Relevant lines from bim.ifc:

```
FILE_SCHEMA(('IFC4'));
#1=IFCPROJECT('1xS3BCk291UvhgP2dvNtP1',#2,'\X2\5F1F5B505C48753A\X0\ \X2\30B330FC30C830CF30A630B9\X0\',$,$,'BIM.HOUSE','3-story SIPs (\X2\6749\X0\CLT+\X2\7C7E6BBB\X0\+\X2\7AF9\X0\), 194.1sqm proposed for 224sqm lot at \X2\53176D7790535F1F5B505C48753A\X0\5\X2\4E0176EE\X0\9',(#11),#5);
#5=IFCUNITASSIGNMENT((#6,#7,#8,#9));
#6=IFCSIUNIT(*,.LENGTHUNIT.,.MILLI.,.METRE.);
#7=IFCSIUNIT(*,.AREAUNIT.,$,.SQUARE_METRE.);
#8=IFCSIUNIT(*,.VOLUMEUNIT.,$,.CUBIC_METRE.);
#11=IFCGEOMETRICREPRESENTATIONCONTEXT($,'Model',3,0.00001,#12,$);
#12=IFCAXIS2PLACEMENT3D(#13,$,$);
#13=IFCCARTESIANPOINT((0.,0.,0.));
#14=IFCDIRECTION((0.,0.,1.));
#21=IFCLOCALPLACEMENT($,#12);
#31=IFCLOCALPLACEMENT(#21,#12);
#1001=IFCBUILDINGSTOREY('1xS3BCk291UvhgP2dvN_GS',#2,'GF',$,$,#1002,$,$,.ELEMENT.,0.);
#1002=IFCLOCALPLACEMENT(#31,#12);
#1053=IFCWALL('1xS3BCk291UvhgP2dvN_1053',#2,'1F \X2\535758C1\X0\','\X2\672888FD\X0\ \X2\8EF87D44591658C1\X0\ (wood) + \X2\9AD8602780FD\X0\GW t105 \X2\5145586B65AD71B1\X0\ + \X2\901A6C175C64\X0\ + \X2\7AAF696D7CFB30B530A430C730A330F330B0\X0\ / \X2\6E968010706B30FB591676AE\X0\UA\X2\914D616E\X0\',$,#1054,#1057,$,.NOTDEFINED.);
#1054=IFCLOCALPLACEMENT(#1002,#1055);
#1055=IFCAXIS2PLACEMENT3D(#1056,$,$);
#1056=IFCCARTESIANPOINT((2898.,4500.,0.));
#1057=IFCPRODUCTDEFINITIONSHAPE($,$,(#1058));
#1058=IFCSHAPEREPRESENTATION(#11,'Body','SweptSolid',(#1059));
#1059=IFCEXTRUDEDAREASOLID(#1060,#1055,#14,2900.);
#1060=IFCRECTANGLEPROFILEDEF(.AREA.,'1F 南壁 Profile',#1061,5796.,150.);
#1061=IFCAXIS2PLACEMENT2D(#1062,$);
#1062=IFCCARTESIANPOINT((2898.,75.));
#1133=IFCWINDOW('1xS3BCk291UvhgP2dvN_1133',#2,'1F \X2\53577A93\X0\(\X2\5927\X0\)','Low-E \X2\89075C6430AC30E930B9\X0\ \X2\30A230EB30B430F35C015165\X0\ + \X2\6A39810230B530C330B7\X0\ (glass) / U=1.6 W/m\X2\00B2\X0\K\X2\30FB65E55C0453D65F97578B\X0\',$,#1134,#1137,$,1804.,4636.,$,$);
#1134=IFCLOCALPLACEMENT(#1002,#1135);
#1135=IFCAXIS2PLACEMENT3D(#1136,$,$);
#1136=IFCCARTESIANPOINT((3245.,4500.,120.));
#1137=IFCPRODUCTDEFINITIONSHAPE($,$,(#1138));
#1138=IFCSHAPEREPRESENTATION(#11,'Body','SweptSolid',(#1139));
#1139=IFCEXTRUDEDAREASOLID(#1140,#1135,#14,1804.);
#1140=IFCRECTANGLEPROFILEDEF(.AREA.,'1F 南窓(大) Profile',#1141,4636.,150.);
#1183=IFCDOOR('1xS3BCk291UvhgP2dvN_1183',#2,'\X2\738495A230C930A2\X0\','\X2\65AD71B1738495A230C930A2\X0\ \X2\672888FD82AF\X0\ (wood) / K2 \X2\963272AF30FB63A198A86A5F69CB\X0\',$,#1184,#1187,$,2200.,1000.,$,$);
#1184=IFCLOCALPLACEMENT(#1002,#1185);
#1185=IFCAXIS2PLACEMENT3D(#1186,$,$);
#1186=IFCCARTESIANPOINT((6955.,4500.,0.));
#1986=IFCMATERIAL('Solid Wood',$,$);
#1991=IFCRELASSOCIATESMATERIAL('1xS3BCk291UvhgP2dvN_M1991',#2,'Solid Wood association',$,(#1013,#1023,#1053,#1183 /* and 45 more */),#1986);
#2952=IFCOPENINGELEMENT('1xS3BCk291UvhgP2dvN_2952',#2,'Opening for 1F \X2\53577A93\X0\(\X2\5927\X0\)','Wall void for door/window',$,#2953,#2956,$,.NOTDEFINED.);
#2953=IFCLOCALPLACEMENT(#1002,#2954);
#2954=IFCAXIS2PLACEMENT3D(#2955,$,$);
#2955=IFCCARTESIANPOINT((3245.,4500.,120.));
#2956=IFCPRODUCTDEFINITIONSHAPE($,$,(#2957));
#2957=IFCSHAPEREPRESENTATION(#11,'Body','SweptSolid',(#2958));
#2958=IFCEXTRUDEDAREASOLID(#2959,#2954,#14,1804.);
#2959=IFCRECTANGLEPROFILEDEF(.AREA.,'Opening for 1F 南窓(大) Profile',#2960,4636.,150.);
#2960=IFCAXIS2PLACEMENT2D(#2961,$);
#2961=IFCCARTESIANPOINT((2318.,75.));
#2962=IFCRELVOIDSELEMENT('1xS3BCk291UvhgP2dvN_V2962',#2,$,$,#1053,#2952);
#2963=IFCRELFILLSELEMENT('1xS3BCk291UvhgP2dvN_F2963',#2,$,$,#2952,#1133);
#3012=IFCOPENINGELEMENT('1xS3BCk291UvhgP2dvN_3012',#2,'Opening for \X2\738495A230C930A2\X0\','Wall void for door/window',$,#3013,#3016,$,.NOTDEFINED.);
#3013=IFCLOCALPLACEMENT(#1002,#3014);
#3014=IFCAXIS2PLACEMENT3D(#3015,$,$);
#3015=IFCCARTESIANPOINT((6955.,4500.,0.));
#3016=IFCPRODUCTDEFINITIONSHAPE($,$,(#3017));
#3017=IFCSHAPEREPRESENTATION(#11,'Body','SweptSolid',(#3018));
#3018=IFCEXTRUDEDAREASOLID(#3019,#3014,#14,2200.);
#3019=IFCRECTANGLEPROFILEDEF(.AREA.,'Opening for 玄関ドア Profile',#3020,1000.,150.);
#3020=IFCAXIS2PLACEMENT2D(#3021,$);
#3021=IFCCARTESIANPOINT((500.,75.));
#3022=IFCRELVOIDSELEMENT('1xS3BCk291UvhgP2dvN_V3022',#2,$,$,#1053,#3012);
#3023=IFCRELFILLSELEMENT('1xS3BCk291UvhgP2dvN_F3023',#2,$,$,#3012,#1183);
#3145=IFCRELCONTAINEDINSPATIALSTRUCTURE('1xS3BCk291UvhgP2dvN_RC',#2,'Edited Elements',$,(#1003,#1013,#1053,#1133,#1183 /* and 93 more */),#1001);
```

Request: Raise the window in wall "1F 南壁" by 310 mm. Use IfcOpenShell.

```python
import numpy as np
import ifcopenshell
import ifcopenshell.api.geometry
import ifcopenshell.util.placement
import ifcopenshell.util.unit

model = ifcopenshell.open("bim.ifc")
unit_scale = ifcopenshell.util.unit.calculate_unit_scale(model)

window = model.by_id(1133)
opening = window.FillsVoids[0].RelatingOpeningElement
dz = 0.31 / unit_scale

shift = np.array([0.0, 0.0, dz])
# The window is not placed relative to its opening, so move both.
for product in (opening, window):
    matrix = ifcopenshell.util.placement.get_local_placement(product.ObjectPlacement)
    matrix[:3, 3] += shift
    ifcopenshell.api.geometry.edit_object_placement(model, product=product, matrix=matrix, is_si=False)

print(f"moved by {dz * unit_scale:+.3f} m")

model.write("bim_edited.ifc")
```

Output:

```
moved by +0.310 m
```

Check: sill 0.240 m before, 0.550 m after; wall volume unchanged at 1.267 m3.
